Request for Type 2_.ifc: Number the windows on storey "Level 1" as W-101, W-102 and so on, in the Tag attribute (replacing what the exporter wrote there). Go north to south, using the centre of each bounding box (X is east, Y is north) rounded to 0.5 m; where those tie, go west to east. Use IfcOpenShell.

First a look at what the model holds.

```python
import ifcopenshell
import ifcopenshell.util.element
import ifcopenshell.util.placement

model = ifcopenshell.open("Type 2_.ifc")
print(model.schema)
storey = next(s for s in model.by_type("IfcBuildingStorey") if s.Name == "Level 1")
windows = [e for e in ifcopenshell.util.element.get_decomposition(storey) if e.is_a("IfcWindow")]
for e in sorted(windows, key=lambda e: e.id()):
    origin = ifcopenshell.util.placement.get_local_placement(e.ObjectPlacement)[:3, 3]
    print(e.id(), e.Tag, e.Name, origin.round(2) + 0.0, sep=" | ")
```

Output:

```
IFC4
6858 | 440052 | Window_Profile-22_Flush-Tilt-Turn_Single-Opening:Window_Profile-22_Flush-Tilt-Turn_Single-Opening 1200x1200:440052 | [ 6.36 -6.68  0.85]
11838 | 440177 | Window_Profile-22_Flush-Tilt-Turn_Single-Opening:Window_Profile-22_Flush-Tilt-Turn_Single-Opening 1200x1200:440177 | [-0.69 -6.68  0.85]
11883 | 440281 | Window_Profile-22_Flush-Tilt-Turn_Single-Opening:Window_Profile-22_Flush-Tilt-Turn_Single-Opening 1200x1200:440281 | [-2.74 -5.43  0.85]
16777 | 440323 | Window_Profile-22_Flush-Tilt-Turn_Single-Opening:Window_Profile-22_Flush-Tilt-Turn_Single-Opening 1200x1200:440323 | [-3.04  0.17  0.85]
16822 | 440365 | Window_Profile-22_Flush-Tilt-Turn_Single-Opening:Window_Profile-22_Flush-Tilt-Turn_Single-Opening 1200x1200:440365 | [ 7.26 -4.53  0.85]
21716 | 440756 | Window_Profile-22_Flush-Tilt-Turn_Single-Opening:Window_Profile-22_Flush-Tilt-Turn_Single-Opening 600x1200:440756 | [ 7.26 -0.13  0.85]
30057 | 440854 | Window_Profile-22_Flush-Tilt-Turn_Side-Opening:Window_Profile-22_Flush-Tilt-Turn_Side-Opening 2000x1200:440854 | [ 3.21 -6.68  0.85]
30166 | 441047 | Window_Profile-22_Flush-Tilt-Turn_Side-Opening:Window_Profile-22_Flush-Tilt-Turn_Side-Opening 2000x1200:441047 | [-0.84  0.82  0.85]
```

```python
import ifcopenshell
import ifcopenshell.geom
import ifcopenshell.util.element
import ifcopenshell.util.shape

model = ifcopenshell.open("Type 2_.ifc")
settings = ifcopenshell.geom.settings()
settings.set("use-world-coords", True)


def centre(element):
    shape = ifcopenshell.geom.create_shape(settings, element)
    return ifcopenshell.util.shape.get_bbox_centroid(shape.geometry)


storey = next(s for s in model.by_type("IfcBuildingStorey") if s.Name == "Level 1")
windows = [e for e in ifcopenshell.util.element.get_decomposition(storey) if e.is_a("IfcWindow")]

# Insertion points can sit at a corner or the storey origin, so sort by the geometry (in metres).
centres = {e: centre(e) for e in windows}
windows.sort(key=lambda e: (-round(centres[e][1] / 0.5), centres[e][0]))

for i, e in enumerate(windows, start=1):
    number = f"W-1{i:02d}"
    e.Tag = number
    print(e.id(), number)

model.write("Type 2__rev.ifc")
```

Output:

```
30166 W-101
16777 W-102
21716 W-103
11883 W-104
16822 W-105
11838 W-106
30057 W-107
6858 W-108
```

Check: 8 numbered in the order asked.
